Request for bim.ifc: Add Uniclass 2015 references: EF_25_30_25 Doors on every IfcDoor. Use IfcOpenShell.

First a look at what the model holds.

```python
import ifcopenshell

model = ifcopenshell.open("bim.ifc")
print(model.schema)
print("classifications:", [c.Name for c in model.by_type("IfcClassification")])
for ifc_class in ("IfcDoor", "IfcRoof", "IfcStair", "IfcWall", "IfcWindow"):
    print(ifc_class, len(model.by_type(ifc_class)))
```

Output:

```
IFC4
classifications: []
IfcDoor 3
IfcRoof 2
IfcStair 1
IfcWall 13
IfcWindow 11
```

```python
import ifcopenshell
import ifcopenshell.api.classification

model = ifcopenshell.open("bim.ifc")

system = ifcopenshell.api.classification.add_classification(model, classification="Uniclass 2015")

codes = {
    "IfcDoor": ("EF_25_30_25", "Doors"),
}
for ifc_class, (code, name) in codes.items():
    products = model.by_type(ifc_class)
    ifcopenshell.api.classification.add_reference(
        model, products=products, classification=system, identification=code, name=name
    )
    print(code, len(products))

model.write("bim_updated.ifc")
```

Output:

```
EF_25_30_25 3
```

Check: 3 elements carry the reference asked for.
